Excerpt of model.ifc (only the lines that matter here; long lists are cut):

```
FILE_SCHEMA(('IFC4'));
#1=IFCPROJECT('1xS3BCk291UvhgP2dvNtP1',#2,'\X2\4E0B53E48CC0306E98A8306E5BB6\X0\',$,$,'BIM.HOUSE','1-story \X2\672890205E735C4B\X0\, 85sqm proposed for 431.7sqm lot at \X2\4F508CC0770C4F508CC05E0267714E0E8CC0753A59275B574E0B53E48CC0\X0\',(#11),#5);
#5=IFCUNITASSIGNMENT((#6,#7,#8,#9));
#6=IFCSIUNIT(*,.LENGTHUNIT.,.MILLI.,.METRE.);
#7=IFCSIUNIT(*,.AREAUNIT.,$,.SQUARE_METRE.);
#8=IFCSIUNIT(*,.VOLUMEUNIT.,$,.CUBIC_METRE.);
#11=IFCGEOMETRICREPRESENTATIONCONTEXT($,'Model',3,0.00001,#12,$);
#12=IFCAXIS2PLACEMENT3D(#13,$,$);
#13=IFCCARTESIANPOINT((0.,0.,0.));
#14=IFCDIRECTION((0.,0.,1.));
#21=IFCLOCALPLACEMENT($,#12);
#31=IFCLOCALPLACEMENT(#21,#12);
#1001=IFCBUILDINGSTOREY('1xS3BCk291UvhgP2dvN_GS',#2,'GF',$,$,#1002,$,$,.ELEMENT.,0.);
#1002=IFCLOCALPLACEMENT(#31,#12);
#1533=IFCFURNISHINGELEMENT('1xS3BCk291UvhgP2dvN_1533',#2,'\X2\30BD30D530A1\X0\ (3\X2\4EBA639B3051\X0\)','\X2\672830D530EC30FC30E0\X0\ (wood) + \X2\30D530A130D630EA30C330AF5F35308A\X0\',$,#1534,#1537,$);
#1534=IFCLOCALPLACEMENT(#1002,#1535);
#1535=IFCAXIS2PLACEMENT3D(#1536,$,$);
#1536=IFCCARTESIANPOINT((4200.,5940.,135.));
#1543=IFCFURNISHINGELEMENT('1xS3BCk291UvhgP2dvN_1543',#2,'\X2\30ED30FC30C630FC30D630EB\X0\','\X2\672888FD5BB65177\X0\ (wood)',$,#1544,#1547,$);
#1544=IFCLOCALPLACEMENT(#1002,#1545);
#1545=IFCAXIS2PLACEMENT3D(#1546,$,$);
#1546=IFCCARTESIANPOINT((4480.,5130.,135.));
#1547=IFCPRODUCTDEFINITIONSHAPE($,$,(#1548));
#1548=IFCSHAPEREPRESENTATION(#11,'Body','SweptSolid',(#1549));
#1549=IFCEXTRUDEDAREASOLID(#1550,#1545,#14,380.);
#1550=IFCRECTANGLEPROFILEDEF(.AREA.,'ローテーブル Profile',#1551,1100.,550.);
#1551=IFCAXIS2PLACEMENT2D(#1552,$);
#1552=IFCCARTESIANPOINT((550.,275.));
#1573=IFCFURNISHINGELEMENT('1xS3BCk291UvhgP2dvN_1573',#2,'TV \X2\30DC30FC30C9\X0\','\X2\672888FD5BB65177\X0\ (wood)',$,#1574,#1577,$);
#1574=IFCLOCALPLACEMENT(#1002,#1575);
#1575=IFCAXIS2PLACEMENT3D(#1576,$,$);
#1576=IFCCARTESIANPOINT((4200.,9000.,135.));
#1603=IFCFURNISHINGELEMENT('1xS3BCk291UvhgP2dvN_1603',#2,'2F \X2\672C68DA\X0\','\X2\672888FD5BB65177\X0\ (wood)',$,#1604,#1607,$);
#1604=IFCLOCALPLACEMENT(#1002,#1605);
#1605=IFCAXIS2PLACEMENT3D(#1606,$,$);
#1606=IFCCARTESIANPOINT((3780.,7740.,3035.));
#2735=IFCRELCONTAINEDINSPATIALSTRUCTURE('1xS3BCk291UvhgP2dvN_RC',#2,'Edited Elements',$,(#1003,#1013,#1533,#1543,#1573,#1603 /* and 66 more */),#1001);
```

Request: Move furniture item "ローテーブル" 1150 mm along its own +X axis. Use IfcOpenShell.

```python
import ifcopenshell
import ifcopenshell.api.geometry
import ifcopenshell.util.placement
import ifcopenshell.util.unit

model = ifcopenshell.open("model.ifc")
unit_scale = ifcopenshell.util.unit.calculate_unit_scale(model)

item = model.by_guid("1xS3BCk291UvhgP2dvN_1543")
matrix = ifcopenshell.util.placement.get_local_placement(item.ObjectPlacement)
matrix[:3, 3] += matrix[:3, 0] * 1.15 / unit_scale
ifcopenshell.api.geometry.edit_object_placement(model, product=item, matrix=matrix, is_si=False)

print(ifcopenshell.util.placement.get_local_placement(item.ObjectPlacement).round(3) + 0.0)

model.write("model_edited.ifc")
```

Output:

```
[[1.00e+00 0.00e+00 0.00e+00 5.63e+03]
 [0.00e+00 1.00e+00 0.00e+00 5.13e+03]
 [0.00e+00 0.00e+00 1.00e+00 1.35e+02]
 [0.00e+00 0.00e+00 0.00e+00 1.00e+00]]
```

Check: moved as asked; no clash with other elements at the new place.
